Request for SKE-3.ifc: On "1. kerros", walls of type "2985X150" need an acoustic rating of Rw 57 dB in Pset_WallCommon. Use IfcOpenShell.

First a look at what the model holds.

```python
import ifcopenshell
import ifcopenshell.util.element

model = ifcopenshell.open("SKE-3.ifc")
print(model.schema)
storey = next(s for s in model.by_type("IfcBuildingStorey") if s.Name == "1. kerros")
walls = [e for e in ifcopenshell.util.element.get_decomposition(storey) if e.is_a("IfcWall")]
seen = {}
for e in walls:
    element_type = ifcopenshell.util.element.get_type(e)
    key = (element_type.Name if element_type != e and element_type else None, ifcopenshell.util.element.get_pset(e, "Pset_WallCommon", "AcousticRating"))
    seen[key] = seen.get(key, 0) + 1
for (name, value), count in sorted(seen.items(), key=str):
    print(count, "x", name, "|", value)
```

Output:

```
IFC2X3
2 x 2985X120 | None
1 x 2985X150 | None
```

```python
import ifcopenshell
import ifcopenshell.api.pset
import ifcopenshell.util.element

model = ifcopenshell.open("SKE-3.ifc")

storey = next(s for s in model.by_type("IfcBuildingStorey") if s.Name == "1. kerros")
walls = [e for e in ifcopenshell.util.element.get_decomposition(storey) if e.is_a("IfcWall")]

count = 0
for e in walls:
    element_type = ifcopenshell.util.element.get_type(e)
    if element_type in (None, e) or element_type.Name != "2985X150":
        continue
    # add_pset returns the element's existing set when there is one.
    pset = ifcopenshell.api.pset.add_pset(model, product=e, name="Pset_WallCommon")
    ifcopenshell.api.pset.edit_pset(model, pset=pset, properties={"AcousticRating": "Rw 57 dB"})
    count += 1

print(count, "walls updated")

model.write("SKE-3_rev.ifc")
```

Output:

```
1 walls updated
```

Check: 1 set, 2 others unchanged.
